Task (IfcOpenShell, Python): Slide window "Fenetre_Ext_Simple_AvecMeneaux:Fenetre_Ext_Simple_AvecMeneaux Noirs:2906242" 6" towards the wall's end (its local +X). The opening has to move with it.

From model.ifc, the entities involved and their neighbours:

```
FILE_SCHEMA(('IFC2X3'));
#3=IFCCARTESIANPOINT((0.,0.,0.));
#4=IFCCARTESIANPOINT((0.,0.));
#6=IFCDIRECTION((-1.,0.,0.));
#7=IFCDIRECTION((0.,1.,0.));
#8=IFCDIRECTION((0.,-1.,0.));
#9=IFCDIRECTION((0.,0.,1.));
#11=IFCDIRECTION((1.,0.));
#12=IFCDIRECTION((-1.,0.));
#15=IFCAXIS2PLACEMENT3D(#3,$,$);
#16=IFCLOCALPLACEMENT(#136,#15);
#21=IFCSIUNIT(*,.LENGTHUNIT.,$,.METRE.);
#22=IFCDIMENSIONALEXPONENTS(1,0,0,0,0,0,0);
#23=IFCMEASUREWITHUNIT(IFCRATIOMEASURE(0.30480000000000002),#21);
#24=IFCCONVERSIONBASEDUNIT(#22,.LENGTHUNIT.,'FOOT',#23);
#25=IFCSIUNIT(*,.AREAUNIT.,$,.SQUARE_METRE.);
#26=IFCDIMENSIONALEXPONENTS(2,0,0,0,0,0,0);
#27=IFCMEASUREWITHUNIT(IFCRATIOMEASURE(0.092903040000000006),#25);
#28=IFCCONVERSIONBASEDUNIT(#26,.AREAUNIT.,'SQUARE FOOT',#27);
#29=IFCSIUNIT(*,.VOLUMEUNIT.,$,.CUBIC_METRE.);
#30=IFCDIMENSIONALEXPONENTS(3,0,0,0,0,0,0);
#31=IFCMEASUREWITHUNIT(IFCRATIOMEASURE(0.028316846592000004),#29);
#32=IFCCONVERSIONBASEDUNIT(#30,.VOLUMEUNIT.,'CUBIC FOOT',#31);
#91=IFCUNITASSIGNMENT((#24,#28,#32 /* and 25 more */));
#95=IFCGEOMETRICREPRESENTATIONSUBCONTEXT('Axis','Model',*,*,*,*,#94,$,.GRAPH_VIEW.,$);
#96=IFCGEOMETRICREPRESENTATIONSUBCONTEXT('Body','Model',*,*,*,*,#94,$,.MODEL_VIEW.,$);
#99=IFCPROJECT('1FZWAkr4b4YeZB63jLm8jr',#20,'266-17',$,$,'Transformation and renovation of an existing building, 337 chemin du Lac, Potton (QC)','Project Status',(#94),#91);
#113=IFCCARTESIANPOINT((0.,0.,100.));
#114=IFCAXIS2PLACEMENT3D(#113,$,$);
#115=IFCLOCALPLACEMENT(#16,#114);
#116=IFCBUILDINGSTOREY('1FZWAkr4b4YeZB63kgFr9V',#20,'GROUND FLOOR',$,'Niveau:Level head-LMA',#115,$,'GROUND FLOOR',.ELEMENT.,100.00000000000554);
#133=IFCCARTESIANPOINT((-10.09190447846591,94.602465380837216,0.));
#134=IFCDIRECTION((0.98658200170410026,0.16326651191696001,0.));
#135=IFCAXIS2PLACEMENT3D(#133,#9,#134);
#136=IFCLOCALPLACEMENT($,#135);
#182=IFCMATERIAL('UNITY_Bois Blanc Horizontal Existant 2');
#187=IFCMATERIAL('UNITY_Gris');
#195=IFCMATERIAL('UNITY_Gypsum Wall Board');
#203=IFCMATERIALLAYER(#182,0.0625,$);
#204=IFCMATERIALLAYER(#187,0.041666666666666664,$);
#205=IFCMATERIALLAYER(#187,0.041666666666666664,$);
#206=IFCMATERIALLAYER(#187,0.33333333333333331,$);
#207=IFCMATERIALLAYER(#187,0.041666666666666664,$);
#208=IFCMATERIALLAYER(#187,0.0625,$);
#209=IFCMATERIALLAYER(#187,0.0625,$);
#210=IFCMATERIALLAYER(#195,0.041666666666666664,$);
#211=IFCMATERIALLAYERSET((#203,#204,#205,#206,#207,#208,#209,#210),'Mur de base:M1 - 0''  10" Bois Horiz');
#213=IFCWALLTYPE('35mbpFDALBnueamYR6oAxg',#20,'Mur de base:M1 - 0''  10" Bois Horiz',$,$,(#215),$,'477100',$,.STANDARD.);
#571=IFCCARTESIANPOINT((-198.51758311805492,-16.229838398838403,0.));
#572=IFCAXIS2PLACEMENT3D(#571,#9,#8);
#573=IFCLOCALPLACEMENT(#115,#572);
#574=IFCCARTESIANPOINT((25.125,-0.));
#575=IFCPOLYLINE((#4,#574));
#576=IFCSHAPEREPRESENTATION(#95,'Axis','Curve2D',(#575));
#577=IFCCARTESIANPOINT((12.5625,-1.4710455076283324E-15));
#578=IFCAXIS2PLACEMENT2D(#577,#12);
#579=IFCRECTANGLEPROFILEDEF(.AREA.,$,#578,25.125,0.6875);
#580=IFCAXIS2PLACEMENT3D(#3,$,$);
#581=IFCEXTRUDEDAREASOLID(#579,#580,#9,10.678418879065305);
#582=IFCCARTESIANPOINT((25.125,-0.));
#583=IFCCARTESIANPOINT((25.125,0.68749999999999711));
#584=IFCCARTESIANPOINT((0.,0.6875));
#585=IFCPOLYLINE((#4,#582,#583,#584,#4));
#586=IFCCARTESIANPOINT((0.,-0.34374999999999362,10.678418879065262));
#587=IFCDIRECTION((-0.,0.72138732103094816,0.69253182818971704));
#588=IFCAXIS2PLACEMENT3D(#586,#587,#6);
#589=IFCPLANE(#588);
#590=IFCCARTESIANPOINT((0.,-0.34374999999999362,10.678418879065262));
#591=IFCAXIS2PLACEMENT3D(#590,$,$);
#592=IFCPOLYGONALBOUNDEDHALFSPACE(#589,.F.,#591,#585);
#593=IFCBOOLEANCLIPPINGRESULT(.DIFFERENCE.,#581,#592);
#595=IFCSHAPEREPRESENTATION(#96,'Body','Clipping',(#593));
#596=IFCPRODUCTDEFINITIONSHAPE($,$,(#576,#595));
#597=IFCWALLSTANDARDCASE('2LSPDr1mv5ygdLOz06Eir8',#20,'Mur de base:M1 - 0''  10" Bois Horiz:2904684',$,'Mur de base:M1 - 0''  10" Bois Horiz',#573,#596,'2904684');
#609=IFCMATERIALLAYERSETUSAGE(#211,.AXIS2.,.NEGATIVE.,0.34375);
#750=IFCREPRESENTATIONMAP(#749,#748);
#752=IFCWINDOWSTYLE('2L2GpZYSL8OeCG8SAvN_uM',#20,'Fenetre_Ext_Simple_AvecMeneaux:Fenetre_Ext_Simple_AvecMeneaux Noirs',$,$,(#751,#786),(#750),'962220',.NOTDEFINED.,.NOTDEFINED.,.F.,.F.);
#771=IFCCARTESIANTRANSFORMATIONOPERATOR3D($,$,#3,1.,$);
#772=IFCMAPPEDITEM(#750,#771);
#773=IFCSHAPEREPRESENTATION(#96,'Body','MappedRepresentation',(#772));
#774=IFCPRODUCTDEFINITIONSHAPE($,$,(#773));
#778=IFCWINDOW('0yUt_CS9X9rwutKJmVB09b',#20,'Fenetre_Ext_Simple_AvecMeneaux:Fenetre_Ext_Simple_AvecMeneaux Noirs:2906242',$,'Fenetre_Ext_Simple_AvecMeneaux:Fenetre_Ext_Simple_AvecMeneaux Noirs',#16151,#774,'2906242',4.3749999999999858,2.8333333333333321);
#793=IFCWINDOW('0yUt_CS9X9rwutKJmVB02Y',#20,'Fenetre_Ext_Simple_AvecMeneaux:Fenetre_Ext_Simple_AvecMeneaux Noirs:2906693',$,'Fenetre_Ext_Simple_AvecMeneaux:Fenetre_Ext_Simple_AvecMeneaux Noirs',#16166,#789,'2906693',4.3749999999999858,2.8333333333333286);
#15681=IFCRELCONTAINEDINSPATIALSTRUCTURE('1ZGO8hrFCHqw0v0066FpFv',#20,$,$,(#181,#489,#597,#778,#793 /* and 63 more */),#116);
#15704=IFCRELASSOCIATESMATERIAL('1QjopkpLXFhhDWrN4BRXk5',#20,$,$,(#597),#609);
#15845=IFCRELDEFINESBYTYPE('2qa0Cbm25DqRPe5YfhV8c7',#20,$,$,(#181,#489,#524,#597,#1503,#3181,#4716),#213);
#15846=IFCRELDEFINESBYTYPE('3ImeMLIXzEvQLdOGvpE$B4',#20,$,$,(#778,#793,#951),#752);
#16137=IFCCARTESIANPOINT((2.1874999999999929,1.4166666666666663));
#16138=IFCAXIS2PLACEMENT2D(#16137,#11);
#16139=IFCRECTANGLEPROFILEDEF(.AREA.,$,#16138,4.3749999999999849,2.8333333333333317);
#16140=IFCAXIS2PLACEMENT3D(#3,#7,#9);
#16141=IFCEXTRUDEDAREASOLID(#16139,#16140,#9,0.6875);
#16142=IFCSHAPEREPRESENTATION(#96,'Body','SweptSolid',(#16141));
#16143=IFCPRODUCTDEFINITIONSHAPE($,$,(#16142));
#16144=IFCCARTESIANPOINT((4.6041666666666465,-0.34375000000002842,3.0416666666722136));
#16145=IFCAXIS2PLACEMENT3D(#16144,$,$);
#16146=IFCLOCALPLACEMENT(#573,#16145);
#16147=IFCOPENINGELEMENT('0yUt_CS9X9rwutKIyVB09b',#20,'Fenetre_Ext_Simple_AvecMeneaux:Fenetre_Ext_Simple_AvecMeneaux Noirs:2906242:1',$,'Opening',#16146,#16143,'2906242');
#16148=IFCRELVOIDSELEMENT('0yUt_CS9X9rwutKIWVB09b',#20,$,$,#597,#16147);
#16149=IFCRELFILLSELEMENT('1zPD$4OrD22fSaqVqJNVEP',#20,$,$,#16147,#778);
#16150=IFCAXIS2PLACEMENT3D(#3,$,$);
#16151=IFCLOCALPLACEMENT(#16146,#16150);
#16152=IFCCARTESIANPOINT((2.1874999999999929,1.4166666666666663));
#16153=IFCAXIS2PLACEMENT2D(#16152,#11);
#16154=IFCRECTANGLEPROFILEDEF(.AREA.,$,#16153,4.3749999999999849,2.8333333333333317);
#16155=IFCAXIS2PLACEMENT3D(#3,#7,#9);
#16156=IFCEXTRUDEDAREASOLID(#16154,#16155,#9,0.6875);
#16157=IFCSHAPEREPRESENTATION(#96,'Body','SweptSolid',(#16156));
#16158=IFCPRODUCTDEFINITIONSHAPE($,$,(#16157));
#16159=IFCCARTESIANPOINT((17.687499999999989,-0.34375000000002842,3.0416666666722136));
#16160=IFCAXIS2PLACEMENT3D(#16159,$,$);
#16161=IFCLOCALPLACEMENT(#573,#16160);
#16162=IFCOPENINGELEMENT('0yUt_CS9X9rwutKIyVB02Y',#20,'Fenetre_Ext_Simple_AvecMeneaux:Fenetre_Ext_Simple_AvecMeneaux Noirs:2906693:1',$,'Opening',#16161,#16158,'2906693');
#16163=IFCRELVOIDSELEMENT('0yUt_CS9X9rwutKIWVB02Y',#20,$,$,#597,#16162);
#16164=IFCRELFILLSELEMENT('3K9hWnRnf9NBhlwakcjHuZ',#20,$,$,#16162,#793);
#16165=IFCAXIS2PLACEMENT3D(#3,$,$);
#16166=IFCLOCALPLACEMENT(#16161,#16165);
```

```python
import ifcopenshell
import ifcopenshell.api.geometry
import ifcopenshell.util.placement
import ifcopenshell.util.unit

model = ifcopenshell.open("model.ifc")
unit_scale = ifcopenshell.util.unit.calculate_unit_scale(model)

window = model.by_id(778)
opening = window.FillsVoids[0].RelatingOpeningElement
wall = opening.VoidsElements[0].RelatingBuildingElement

wall_matrix = ifcopenshell.util.placement.get_local_placement(wall.ObjectPlacement)
shift = wall_matrix[:3, 0] * 6 * 0.0254 / unit_scale
before = ifcopenshell.util.placement.get_local_placement(window.ObjectPlacement)[:3, 3].copy()

# The window is placed relative to its opening, so it follows when the opening moves.
matrix = ifcopenshell.util.placement.get_local_placement(opening.ObjectPlacement)
matrix[:3, 3] += shift
ifcopenshell.api.geometry.edit_object_placement(
    model, product=opening, matrix=matrix, is_si=False, should_transform_children=True
)

after = ifcopenshell.util.placement.get_local_placement(window.ObjectPlacement)[:3, 3]
print("window moved by", (after - before).round(3) + 0.0)

model.write("model_rev.ifc")
```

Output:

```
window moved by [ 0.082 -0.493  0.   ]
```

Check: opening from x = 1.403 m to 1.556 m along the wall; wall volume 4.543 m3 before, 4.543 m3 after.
